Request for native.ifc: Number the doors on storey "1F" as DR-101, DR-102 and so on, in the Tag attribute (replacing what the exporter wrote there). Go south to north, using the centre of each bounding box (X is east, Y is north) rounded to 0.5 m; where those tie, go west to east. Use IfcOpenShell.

First a look at what the model holds.

```python
import ifcopenshell
import ifcopenshell.util.element
import ifcopenshell.util.placement

model = ifcopenshell.open("native.ifc")
print(model.schema)
storey = next(s for s in model.by_type("IfcBuildingStorey") if s.Name == "1F")
doors = [e for e in ifcopenshell.util.element.get_decomposition(storey) if e.is_a("IfcDoor")]
for e in sorted(doors, key=lambda e: e.id()):
    origin = ifcopenshell.util.placement.get_local_placement(e.ObjectPlacement)[:3, 3]
    print(e.id(), e.Tag, e.Name, origin.round(2) + 0.0, sep=" | ")
```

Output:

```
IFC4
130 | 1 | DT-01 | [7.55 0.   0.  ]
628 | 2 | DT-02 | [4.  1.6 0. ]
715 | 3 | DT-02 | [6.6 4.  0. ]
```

```python
import ifcopenshell
import ifcopenshell.geom
import ifcopenshell.util.element
import ifcopenshell.util.shape

model = ifcopenshell.open("native.ifc")
settings = ifcopenshell.geom.settings()
settings.set("use-world-coords", True)


def centre(element):
    shape = ifcopenshell.geom.create_shape(settings, element)
    return ifcopenshell.util.shape.get_bbox_centroid(shape.geometry)


storey = next(s for s in model.by_type("IfcBuildingStorey") if s.Name == "1F")
doors = [e for e in ifcopenshell.util.element.get_decomposition(storey) if e.is_a("IfcDoor")]

# Insertion points can sit at a corner or the storey origin, so sort by the geometry (in metres).
centres = {e: centre(e) for e in doors}
doors.sort(key=lambda e: (round(centres[e][1] / 0.5), centres[e][0]))

for i, e in enumerate(doors, start=1):
    number = f"DR-1{i:02d}"
    e.Tag = number
    print(e.id(), number)

model.write("native_v2.ifc")
```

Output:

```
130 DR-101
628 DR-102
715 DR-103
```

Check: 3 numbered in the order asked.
